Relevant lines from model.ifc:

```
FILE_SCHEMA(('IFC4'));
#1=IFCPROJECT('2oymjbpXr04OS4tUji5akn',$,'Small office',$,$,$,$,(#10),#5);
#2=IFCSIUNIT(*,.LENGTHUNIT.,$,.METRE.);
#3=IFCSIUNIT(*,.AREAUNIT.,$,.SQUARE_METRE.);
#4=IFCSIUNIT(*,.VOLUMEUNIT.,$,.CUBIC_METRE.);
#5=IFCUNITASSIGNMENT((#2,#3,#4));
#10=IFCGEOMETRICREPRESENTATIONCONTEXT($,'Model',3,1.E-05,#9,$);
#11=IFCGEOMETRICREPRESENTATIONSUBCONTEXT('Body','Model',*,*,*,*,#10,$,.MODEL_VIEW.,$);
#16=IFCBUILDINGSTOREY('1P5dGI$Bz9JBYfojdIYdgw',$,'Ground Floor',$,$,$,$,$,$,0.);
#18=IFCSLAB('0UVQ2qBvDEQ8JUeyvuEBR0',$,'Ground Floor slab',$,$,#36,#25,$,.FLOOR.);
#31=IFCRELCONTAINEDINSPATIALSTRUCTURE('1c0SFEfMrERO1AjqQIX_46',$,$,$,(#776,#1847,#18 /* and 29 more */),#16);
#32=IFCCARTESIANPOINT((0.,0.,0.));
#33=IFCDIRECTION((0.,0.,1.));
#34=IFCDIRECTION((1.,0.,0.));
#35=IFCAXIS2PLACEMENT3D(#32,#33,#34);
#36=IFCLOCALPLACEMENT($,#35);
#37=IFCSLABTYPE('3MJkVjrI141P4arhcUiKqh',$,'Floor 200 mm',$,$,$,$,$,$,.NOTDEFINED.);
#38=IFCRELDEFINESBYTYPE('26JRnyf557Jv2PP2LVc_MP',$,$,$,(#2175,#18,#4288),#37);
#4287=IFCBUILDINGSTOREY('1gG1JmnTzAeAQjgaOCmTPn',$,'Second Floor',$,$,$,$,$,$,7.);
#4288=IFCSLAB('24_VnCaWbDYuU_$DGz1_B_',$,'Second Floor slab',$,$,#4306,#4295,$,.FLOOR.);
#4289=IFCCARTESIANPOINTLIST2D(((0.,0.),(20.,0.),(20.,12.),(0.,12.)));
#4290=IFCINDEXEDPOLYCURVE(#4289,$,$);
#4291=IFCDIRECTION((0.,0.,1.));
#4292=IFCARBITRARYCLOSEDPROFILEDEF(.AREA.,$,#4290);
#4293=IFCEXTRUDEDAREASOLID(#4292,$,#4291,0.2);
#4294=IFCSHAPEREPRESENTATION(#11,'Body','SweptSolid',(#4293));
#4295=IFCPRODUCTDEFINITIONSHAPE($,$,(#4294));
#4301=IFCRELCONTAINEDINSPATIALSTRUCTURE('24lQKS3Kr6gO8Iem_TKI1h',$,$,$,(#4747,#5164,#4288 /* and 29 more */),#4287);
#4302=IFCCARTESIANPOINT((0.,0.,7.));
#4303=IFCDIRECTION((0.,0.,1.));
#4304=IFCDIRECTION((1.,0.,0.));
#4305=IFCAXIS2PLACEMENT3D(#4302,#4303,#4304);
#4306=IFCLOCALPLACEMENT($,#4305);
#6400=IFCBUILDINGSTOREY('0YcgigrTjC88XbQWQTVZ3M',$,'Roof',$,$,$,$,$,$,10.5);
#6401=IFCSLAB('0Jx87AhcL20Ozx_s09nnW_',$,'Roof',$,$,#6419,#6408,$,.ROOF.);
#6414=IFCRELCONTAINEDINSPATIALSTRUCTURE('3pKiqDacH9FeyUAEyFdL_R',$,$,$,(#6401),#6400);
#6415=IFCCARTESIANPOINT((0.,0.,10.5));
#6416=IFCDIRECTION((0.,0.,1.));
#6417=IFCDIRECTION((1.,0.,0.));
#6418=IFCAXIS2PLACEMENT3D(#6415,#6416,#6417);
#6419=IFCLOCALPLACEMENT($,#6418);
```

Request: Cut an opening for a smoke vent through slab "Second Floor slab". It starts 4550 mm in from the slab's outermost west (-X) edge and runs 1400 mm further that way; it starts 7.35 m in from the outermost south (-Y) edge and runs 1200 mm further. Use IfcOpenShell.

```python
import numpy as np
import ifcopenshell
import ifcopenshell.api.feature
import ifcopenshell.api.geometry
import ifcopenshell.api.root
import ifcopenshell.geom
import ifcopenshell.util.placement
import ifcopenshell.util.representation
import ifcopenshell.util.shape
import ifcopenshell.util.unit

model = ifcopenshell.open("model.ifc")
unit_scale = ifcopenshell.util.unit.calculate_unit_scale(model)
settings = ifcopenshell.geom.settings()


def volume(element):
    """Net volume in cubic metres, openings subtracted."""
    shape = ifcopenshell.geom.create_shape(settings, element)
    return ifcopenshell.util.shape.get_volume(shape.geometry)


slab = model.by_guid("24_VnCaWbDYuU_$DGz1_B_")
before = volume(slab)

# Extent in the slab's own axes, in metres. The edges named are its -X and -Y sides.
slab_shape = ifcopenshell.geom.create_shape(settings, slab)
vertices = ifcopenshell.util.shape.get_vertices(slab_shape.geometry)
x_min, y_min, bottom = vertices.min(axis=0)
top = vertices[:, 2].max()

opening = ifcopenshell.api.root.create_entity(model, ifc_class="IfcOpeningElement", name="Smoke vent opening", predefined_type="OPENING")
context = ifcopenshell.util.representation.get_context(model, "Model", "Body", "MODEL_VIEW")
width, depth = 1.4, 1.2
outline = [(0.0, 0.0), (width, 0.0), (width, depth), (0.0, depth), (0.0, 0.0)]
# Overshoot both faces by 50 mm so the cut is clean.
shape = ifcopenshell.api.geometry.add_slab_representation(
    model, context=context, depth=top - bottom + 0.1, polyline=outline
)
ifcopenshell.api.geometry.assign_representation(model, product=opening, representation=shape)

matrix = ifcopenshell.util.placement.get_local_placement(slab.ObjectPlacement)
matrix[:, 3] = matrix @ np.append(np.array([x_min + 4.55, y_min + 7.35, bottom - 0.05]) / unit_scale, 1.0)
ifcopenshell.api.geometry.edit_object_placement(model, product=opening, matrix=matrix, is_si=False)
ifcopenshell.api.feature.add_feature(model, feature=opening, element=slab)

after = volume(slab)

print(f"slab volume {before:.3f} -> {after:.3f} m3")

model.write("model_updated.ifc")
```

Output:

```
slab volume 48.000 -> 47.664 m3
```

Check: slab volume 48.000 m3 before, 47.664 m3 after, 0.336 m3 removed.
